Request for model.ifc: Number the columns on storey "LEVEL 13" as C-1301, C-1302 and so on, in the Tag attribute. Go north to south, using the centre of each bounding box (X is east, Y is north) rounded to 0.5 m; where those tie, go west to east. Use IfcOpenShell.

First a look at what the model holds.

```python
import ifcopenshell
import ifcopenshell.util.element
import ifcopenshell.util.placement

model = ifcopenshell.open("model.ifc")
print(model.schema)
storey = next(s for s in model.by_type("IfcBuildingStorey") if s.Name == "LEVEL 13")
columns = [e for e in ifcopenshell.util.element.get_decomposition(storey) if e.is_a("IfcColumn")]
for e in sorted(columns, key=lambda e: e.id()):
    origin = ifcopenshell.util.placement.get_local_placement(e.ObjectPlacement)[:3, 3]
    print(e.id(), e.Tag, e.Name, origin.round(2) + 0.0, sep=" | ")
```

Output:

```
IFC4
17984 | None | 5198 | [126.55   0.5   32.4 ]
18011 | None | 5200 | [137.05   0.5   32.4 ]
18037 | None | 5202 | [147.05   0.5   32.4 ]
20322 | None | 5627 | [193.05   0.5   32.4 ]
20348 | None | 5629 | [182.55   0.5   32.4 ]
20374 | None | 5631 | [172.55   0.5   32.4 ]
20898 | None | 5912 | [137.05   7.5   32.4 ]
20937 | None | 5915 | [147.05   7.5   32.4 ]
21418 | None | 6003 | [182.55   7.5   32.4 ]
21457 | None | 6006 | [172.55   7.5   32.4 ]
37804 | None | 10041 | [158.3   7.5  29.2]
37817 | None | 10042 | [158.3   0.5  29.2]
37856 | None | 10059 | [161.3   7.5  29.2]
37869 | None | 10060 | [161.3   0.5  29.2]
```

```python
import ifcopenshell
import ifcopenshell.geom
import ifcopenshell.util.element
import ifcopenshell.util.shape

model = ifcopenshell.open("model.ifc")
settings = ifcopenshell.geom.settings()
settings.set("use-world-coords", True)


def centre(element):
    shape = ifcopenshell.geom.create_shape(settings, element)
    return ifcopenshell.util.shape.get_bbox_centroid(shape.geometry)


storey = next(s for s in model.by_type("IfcBuildingStorey") if s.Name == "LEVEL 13")
columns = [e for e in ifcopenshell.util.element.get_decomposition(storey) if e.is_a("IfcColumn")]

# Insertion points can sit at a corner or the storey origin, so sort by the geometry (in metres).
centres = {e: centre(e) for e in columns}
columns.sort(key=lambda e: (-round(centres[e][1] / 0.5), centres[e][0]))

for i, e in enumerate(columns, start=1):
    number = f"C-13{i:02d}"
    e.Tag = number
    print(e.id(), number)

model.write("model_edited.ifc")
```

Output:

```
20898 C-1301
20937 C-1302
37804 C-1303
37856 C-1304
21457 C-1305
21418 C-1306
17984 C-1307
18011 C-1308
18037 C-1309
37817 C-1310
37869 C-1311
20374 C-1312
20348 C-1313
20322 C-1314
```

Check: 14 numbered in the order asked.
